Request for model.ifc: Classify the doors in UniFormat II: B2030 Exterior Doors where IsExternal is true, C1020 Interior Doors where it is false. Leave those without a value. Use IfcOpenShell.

First a look at what the model holds.

```python
import ifcopenshell
import ifcopenshell.util.element

model = ifcopenshell.open("model.ifc")
print(model.schema)
print("classifications:", [c.Name for c in model.by_type("IfcClassification")])
values = [ifcopenshell.util.element.get_pset(e, "Pset_DoorCommon", "IsExternal") for e in model.by_type("IfcDoor")]
for value in (True, False, None):
    print("IsExternal", value, values.count(value))
```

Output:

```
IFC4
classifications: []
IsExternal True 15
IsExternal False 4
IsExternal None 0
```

```python
import ifcopenshell
import ifcopenshell.api.classification
import ifcopenshell.util.element

model = ifcopenshell.open("model.ifc")

system = ifcopenshell.api.classification.add_classification(model, classification="UniFormat II")

doors = model.by_type("IfcDoor")
external = {e: ifcopenshell.util.element.get_pset(e, "Pset_DoorCommon", "IsExternal") for e in doors}
for flag, code, name in ((True, "B2030", "Exterior Doors"), (False, "C1020", "Interior Doors")):
    products = [e for e in doors if external[e] is flag]
    ifcopenshell.api.classification.add_reference(
        model, products=products, classification=system, identification=code, name=name
    )
    print(code, len(products))

model.write("model_updated.ifc")
```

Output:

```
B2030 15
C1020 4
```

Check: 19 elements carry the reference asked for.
